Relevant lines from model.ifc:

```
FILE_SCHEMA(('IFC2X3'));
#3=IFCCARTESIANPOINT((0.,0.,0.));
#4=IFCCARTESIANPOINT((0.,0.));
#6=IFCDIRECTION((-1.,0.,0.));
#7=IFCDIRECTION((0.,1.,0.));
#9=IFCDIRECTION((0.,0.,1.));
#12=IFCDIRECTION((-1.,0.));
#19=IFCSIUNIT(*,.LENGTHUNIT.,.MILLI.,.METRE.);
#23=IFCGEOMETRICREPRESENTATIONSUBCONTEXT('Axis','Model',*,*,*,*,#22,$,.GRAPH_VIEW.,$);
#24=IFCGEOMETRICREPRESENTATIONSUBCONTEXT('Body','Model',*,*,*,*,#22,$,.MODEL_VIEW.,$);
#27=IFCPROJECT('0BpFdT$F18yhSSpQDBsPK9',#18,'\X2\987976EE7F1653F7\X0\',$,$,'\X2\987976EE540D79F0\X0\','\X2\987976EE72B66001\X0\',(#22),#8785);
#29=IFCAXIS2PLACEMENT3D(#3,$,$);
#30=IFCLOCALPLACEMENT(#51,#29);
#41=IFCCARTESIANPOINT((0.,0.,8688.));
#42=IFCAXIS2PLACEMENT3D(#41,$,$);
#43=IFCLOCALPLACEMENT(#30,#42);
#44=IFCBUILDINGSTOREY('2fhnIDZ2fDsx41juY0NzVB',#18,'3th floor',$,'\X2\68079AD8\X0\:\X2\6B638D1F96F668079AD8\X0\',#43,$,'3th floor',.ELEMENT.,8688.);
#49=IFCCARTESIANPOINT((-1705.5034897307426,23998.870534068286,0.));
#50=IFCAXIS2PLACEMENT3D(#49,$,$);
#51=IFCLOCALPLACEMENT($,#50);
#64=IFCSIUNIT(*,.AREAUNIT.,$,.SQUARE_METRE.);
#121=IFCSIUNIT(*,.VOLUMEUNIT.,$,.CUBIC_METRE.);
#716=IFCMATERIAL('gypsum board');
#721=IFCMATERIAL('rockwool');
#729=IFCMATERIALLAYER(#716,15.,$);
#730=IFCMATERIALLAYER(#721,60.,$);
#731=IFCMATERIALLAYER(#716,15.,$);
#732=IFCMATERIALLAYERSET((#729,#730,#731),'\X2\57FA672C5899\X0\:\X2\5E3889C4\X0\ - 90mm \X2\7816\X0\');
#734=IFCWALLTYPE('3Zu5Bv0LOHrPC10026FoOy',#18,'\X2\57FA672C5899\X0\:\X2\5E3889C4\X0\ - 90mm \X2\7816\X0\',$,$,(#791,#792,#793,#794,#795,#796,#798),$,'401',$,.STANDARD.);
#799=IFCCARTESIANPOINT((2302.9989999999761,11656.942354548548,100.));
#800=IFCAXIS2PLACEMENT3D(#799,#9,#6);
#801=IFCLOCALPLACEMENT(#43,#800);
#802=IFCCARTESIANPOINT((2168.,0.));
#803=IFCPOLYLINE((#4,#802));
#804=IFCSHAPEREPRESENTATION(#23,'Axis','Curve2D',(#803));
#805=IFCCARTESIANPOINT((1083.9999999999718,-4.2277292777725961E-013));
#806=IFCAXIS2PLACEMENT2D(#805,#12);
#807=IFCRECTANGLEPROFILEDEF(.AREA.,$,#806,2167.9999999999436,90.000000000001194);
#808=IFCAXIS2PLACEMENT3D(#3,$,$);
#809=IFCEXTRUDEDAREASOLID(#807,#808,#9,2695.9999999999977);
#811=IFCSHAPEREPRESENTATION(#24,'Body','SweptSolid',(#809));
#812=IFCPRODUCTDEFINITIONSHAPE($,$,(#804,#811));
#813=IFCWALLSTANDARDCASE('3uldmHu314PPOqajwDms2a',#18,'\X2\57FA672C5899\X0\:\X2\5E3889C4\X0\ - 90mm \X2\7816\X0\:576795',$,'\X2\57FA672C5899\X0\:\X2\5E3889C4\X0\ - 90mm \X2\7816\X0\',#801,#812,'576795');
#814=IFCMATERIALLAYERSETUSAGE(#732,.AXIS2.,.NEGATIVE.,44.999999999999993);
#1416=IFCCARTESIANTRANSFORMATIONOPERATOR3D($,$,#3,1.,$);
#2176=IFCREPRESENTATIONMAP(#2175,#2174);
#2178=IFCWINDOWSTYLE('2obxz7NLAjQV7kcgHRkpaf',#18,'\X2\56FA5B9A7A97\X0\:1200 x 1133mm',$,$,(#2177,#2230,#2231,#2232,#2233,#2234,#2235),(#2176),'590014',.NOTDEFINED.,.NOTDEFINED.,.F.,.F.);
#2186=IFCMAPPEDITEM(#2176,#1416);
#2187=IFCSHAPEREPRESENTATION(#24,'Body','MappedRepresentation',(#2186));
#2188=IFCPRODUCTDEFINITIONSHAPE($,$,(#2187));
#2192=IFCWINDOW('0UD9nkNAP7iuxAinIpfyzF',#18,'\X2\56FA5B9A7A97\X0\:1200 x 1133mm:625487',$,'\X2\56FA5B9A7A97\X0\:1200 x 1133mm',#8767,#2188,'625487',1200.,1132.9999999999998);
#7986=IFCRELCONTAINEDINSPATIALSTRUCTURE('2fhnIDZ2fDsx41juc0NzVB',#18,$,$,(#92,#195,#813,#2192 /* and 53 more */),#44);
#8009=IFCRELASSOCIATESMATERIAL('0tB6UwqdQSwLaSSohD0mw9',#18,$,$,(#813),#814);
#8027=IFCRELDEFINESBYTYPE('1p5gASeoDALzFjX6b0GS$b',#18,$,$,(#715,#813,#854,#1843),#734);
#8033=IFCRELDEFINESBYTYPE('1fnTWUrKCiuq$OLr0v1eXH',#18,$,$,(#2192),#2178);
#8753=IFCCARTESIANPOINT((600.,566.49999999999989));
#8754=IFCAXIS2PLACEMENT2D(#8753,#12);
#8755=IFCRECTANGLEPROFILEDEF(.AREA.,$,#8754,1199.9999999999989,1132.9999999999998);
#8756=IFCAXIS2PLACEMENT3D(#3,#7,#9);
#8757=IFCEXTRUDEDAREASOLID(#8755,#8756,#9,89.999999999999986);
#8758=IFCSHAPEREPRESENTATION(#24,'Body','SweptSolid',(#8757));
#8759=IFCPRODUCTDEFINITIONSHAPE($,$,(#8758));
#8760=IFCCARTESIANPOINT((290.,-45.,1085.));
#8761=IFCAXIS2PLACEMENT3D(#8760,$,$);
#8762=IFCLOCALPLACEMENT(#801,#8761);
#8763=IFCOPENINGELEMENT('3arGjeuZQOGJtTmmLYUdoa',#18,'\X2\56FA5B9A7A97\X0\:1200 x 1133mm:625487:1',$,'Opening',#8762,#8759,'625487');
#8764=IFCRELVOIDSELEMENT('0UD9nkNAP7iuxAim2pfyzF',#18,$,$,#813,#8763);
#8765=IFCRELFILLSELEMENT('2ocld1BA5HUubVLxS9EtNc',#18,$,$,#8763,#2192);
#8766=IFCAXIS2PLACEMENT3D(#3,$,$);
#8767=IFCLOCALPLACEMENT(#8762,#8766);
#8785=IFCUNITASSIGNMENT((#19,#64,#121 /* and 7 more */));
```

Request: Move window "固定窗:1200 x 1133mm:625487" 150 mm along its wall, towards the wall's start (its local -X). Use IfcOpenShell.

```python
import ifcopenshell
import ifcopenshell.api.geometry
import ifcopenshell.util.placement

model = ifcopenshell.open("model.ifc")

window = model.by_guid("0UD9nkNAP7iuxAinIpfyzF")
opening = window.FillsVoids[0].RelatingOpeningElement
wall = opening.VoidsElements[0].RelatingBuildingElement

wall_matrix = ifcopenshell.util.placement.get_local_placement(wall.ObjectPlacement)
shift = wall_matrix[:3, 0] * -150.0
before = ifcopenshell.util.placement.get_local_placement(window.ObjectPlacement)[:3, 3].copy()

# The window is placed relative to its opening, so it follows when the opening moves.
matrix = ifcopenshell.util.placement.get_local_placement(opening.ObjectPlacement)
matrix[:3, 3] += shift
ifcopenshell.api.geometry.edit_object_placement(
    model, product=opening, matrix=matrix, is_si=False, should_transform_children=True
)

after = ifcopenshell.util.placement.get_local_placement(window.ObjectPlacement)[:3, 3]
print("window moved by", (after - before).round(3) + 0.0)

model.write("model_rev.ifc")
```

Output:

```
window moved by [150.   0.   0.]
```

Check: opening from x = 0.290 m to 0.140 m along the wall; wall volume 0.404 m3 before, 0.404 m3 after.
